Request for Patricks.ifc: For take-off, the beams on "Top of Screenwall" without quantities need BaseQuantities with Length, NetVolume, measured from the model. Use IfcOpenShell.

First a look at what the model holds.

```python
import ifcopenshell
import ifcopenshell.util.element
import ifcopenshell.util.unit

model = ifcopenshell.open("Patricks.ifc")
print(model.schema)
for unit_type in ("LENGTHUNIT", "AREAUNIT", "VOLUMEUNIT"):
    print(unit_type, ifcopenshell.util.unit.calculate_unit_scale(model, unit_type))
storey = next(s for s in model.by_type("IfcBuildingStorey") if s.Name == "Top of Screenwall")
beams = [e for e in ifcopenshell.util.element.get_decomposition(storey) if e.is_a("IfcBeam")]
for e in sorted(beams, key=lambda e: e.id()):
    print(e.id(), e.is_a(), e.Name, list(ifcopenshell.util.element.get_psets(e, qtos_only=True)), sep=" | ")
```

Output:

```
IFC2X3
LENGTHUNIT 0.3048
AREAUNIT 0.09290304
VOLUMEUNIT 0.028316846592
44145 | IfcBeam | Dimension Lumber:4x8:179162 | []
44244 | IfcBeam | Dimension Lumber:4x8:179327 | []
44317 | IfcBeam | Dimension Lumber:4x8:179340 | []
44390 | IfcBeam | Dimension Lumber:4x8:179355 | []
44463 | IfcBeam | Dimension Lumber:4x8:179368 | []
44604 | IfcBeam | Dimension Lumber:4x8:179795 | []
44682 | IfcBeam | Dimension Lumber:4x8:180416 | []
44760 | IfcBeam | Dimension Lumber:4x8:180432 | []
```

```python
import ifcopenshell
import ifcopenshell.api.pset
import ifcopenshell.geom
import ifcopenshell.util.element
import ifcopenshell.util.shape
import ifcopenshell.util.unit

model = ifcopenshell.open("Patricks.ifc")
unit_scale = ifcopenshell.util.unit.calculate_unit_scale(model)
volume_scale = ifcopenshell.util.unit.calculate_unit_scale(model, "VOLUMEUNIT")
settings = ifcopenshell.geom.settings()

storey = next(s for s in model.by_type("IfcBuildingStorey") if s.Name == "Top of Screenwall")
beams = [e for e in ifcopenshell.util.element.get_decomposition(storey) if e.is_a("IfcBeam")]

for e in sorted(beams, key=lambda e: e.id()):
    if ifcopenshell.util.element.get_psets(e, qtos_only=True, should_inherit=False):
        continue
    # Geometry comes back in metres, in the element's own axes.
    shape = ifcopenshell.geom.create_shape(settings, e)
    values = {
        "Length": ifcopenshell.util.shape.get_max_xyz(shape.geometry) / unit_scale,
        "NetVolume": ifcopenshell.util.shape.get_volume(shape.geometry) / volume_scale,
    }
    qto = ifcopenshell.api.pset.add_qto(model, product=e, name="BaseQuantities")
    ifcopenshell.api.pset.edit_qto(model, qto=qto, properties=values)
    print(e.id(), {k: round(v, 3) for k, v in values.items()})

model.write("Patricks_rev.ifc")
```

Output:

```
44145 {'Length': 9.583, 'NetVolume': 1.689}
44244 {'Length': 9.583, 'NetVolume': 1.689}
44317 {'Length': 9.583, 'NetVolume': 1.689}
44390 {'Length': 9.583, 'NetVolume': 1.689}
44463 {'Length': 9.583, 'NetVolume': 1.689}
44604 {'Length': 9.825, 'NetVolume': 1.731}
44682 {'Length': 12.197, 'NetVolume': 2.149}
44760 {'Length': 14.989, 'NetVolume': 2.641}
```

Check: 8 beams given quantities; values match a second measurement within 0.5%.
